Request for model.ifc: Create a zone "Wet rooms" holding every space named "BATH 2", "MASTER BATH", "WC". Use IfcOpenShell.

First a look at what the model holds.

```python
import ifcopenshell

model = ifcopenshell.open("model.ifc")
print(model.schema)
seen = {}
for space in model.by_type("IfcSpace"):
    seen[space.LongName] = seen.get(space.LongName, 0) + 1
for name, count in sorted(seen.items(), key=str):
    print(count, "x", name)
print("zones:", [z.Name for z in model.by_type("IfcZone")][:20])
```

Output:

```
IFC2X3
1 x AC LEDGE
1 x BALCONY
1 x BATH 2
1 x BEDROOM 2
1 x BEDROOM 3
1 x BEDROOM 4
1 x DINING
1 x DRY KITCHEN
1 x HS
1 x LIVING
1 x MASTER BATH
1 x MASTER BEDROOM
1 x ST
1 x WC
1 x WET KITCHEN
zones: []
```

```python
import ifcopenshell
import ifcopenshell.api.group
import ifcopenshell.api.root

model = ifcopenshell.open("model.ifc")

names = {"BATH 2", "MASTER BATH", "WC"}
spaces = [s for s in model.by_type("IfcSpace") if s.LongName in names]

zone = ifcopenshell.api.root.create_entity(model, ifc_class="IfcZone", name="Wet rooms")
ifcopenshell.api.group.assign_group(model, products=spaces, group=zone)
print(len(spaces), "spaces in", zone.Name)

model.write("model_updated.ifc")
```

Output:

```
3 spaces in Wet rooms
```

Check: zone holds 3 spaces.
